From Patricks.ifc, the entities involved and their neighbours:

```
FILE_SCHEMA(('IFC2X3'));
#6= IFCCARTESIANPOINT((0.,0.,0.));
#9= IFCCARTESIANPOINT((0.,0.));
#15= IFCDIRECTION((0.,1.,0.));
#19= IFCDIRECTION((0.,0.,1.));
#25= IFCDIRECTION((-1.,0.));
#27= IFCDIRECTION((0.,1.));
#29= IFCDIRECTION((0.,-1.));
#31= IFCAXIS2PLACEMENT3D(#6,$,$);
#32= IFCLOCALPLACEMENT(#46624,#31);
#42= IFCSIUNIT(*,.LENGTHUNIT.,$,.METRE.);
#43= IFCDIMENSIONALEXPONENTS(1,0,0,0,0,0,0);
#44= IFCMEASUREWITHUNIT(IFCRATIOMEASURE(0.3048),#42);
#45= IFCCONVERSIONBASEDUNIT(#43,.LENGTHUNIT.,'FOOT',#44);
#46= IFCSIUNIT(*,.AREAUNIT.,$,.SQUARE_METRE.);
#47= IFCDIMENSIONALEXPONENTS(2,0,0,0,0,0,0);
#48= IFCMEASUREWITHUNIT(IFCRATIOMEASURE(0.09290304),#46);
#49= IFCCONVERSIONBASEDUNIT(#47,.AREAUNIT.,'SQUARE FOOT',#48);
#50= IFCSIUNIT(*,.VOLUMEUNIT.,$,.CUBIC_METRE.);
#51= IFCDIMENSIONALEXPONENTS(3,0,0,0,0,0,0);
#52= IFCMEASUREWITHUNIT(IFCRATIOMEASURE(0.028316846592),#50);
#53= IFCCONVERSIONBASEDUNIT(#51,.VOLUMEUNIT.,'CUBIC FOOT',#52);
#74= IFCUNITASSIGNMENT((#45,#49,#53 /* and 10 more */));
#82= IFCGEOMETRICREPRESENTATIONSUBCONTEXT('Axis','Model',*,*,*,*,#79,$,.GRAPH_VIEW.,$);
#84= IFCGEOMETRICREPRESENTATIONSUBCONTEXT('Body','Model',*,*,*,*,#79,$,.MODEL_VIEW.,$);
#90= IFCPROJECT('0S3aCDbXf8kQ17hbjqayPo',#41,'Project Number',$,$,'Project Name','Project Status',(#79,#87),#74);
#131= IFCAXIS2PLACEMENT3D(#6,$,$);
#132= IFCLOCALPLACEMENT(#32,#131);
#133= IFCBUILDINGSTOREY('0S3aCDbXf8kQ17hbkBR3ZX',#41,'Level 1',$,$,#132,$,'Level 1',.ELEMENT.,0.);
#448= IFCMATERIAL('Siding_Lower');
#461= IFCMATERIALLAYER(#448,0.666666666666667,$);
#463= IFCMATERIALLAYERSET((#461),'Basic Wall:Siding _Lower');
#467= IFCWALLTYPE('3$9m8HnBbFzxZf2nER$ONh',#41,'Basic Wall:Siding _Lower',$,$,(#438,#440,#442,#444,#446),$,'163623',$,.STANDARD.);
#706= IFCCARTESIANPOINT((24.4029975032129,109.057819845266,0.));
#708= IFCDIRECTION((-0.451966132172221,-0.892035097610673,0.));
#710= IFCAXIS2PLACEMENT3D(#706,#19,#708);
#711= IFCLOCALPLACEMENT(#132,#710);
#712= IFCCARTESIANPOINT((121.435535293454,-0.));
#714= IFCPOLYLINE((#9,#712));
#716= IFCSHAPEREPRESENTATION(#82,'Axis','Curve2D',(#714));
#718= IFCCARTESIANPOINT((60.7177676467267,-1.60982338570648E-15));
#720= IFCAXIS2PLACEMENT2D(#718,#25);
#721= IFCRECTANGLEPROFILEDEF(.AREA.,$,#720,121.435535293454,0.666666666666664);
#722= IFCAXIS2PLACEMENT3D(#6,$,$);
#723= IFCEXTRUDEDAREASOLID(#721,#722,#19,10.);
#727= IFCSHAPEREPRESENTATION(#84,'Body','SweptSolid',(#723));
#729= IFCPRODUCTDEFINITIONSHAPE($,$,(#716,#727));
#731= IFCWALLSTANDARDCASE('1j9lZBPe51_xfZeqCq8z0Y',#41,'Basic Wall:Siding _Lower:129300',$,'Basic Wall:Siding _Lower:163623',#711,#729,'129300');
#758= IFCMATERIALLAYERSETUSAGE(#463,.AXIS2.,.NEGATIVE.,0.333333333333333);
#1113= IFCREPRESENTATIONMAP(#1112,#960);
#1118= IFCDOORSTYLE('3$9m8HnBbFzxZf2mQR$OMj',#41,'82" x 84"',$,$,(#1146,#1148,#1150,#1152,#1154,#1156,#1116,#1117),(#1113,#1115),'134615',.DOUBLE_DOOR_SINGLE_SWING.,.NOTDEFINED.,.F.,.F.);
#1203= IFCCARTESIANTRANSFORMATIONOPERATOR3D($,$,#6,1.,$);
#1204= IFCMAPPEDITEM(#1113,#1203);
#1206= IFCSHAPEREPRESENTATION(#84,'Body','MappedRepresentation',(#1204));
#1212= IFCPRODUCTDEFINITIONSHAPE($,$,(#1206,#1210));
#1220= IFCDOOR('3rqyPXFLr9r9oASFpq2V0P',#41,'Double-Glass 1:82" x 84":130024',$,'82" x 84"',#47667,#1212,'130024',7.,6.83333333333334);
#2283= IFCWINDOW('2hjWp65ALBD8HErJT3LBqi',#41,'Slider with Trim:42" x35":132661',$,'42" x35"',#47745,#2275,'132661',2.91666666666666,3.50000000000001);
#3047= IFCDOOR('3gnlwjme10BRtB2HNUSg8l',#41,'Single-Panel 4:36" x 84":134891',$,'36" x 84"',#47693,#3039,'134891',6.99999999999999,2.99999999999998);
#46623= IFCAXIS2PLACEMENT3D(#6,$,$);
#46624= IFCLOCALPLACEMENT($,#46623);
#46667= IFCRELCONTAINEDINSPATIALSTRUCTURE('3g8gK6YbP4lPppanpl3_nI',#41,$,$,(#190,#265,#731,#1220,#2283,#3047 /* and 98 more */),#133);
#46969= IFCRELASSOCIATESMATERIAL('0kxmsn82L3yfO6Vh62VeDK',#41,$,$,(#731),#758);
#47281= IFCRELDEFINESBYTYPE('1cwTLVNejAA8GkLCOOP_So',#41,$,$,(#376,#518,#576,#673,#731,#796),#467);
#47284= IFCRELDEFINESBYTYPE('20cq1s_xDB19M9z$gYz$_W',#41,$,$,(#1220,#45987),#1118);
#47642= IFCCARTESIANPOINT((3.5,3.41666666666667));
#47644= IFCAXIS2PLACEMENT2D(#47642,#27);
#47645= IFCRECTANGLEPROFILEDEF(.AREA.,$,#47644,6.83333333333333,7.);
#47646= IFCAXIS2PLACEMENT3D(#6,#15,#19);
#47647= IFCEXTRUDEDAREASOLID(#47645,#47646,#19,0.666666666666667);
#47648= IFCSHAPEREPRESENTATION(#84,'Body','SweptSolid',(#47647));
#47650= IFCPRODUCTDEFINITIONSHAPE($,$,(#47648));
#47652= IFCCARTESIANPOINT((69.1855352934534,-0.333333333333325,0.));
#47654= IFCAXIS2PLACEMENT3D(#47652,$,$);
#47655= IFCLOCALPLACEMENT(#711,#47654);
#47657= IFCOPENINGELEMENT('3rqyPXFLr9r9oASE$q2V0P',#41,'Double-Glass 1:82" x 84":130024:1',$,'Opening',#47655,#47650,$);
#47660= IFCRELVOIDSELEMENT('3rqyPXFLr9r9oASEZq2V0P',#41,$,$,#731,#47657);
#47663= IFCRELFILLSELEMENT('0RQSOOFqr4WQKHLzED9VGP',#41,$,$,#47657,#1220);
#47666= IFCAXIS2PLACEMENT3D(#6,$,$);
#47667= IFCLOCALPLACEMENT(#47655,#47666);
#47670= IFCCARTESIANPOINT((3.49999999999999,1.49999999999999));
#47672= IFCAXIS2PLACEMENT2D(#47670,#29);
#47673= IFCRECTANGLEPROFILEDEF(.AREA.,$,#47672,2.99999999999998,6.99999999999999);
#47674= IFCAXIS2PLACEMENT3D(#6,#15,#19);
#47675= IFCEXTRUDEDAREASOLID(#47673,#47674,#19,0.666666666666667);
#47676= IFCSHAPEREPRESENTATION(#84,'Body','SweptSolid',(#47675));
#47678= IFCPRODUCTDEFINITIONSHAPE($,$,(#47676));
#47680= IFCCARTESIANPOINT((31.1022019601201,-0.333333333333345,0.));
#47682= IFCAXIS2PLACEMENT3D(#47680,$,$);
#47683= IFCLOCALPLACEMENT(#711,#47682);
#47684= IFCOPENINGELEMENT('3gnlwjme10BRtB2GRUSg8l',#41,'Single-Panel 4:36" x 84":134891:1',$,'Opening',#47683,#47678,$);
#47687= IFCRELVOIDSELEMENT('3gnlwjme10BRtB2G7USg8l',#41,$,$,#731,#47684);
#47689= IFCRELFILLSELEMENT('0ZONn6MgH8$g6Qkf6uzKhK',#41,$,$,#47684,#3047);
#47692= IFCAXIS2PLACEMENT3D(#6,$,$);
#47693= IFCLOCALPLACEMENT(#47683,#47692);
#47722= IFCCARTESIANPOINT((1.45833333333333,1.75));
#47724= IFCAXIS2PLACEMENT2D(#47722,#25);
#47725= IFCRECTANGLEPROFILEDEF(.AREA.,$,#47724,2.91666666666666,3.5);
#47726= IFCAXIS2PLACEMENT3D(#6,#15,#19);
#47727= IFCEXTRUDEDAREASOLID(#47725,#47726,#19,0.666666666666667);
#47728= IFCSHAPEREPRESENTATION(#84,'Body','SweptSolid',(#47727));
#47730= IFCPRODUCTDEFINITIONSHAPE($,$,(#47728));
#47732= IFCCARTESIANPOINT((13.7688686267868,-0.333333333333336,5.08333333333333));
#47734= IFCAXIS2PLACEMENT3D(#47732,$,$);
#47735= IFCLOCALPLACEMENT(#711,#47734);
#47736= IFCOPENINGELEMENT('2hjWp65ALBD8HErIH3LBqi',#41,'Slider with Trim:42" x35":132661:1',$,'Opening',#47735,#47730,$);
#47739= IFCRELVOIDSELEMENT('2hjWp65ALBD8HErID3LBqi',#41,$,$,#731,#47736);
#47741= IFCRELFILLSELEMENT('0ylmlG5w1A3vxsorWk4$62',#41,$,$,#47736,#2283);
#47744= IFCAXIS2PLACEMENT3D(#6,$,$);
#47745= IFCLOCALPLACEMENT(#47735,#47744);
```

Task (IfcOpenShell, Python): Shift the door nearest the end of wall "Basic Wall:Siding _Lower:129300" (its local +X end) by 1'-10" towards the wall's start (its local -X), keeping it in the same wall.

```python
import ifcopenshell
import ifcopenshell.api.geometry
import ifcopenshell.util.placement
import ifcopenshell.util.unit

model = ifcopenshell.open("Patricks.ifc")
unit_scale = ifcopenshell.util.unit.calculate_unit_scale(model)

door = model.by_guid("3rqyPXFLr9r9oASFpq2V0P")
opening = door.FillsVoids[0].RelatingOpeningElement
wall = opening.VoidsElements[0].RelatingBuildingElement

wall_matrix = ifcopenshell.util.placement.get_local_placement(wall.ObjectPlacement)
shift = wall_matrix[:3, 0] * -22 * 0.0254 / unit_scale
before = ifcopenshell.util.placement.get_local_placement(door.ObjectPlacement)[:3, 3].copy()

# The door is placed relative to its opening, so it follows when the opening moves.
matrix = ifcopenshell.util.placement.get_local_placement(opening.ObjectPlacement)
matrix[:3, 3] += shift
ifcopenshell.api.geometry.edit_object_placement(
    model, product=opening, matrix=matrix, is_si=False, should_transform_children=True
)

after = ifcopenshell.util.placement.get_local_placement(door.ObjectPlacement)[:3, 3]
print("door moved by", (after - before).round(3) + 0.0)

model.write("Patricks_edited.ifc")
```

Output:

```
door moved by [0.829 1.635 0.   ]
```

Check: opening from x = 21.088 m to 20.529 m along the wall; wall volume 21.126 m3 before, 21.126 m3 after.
